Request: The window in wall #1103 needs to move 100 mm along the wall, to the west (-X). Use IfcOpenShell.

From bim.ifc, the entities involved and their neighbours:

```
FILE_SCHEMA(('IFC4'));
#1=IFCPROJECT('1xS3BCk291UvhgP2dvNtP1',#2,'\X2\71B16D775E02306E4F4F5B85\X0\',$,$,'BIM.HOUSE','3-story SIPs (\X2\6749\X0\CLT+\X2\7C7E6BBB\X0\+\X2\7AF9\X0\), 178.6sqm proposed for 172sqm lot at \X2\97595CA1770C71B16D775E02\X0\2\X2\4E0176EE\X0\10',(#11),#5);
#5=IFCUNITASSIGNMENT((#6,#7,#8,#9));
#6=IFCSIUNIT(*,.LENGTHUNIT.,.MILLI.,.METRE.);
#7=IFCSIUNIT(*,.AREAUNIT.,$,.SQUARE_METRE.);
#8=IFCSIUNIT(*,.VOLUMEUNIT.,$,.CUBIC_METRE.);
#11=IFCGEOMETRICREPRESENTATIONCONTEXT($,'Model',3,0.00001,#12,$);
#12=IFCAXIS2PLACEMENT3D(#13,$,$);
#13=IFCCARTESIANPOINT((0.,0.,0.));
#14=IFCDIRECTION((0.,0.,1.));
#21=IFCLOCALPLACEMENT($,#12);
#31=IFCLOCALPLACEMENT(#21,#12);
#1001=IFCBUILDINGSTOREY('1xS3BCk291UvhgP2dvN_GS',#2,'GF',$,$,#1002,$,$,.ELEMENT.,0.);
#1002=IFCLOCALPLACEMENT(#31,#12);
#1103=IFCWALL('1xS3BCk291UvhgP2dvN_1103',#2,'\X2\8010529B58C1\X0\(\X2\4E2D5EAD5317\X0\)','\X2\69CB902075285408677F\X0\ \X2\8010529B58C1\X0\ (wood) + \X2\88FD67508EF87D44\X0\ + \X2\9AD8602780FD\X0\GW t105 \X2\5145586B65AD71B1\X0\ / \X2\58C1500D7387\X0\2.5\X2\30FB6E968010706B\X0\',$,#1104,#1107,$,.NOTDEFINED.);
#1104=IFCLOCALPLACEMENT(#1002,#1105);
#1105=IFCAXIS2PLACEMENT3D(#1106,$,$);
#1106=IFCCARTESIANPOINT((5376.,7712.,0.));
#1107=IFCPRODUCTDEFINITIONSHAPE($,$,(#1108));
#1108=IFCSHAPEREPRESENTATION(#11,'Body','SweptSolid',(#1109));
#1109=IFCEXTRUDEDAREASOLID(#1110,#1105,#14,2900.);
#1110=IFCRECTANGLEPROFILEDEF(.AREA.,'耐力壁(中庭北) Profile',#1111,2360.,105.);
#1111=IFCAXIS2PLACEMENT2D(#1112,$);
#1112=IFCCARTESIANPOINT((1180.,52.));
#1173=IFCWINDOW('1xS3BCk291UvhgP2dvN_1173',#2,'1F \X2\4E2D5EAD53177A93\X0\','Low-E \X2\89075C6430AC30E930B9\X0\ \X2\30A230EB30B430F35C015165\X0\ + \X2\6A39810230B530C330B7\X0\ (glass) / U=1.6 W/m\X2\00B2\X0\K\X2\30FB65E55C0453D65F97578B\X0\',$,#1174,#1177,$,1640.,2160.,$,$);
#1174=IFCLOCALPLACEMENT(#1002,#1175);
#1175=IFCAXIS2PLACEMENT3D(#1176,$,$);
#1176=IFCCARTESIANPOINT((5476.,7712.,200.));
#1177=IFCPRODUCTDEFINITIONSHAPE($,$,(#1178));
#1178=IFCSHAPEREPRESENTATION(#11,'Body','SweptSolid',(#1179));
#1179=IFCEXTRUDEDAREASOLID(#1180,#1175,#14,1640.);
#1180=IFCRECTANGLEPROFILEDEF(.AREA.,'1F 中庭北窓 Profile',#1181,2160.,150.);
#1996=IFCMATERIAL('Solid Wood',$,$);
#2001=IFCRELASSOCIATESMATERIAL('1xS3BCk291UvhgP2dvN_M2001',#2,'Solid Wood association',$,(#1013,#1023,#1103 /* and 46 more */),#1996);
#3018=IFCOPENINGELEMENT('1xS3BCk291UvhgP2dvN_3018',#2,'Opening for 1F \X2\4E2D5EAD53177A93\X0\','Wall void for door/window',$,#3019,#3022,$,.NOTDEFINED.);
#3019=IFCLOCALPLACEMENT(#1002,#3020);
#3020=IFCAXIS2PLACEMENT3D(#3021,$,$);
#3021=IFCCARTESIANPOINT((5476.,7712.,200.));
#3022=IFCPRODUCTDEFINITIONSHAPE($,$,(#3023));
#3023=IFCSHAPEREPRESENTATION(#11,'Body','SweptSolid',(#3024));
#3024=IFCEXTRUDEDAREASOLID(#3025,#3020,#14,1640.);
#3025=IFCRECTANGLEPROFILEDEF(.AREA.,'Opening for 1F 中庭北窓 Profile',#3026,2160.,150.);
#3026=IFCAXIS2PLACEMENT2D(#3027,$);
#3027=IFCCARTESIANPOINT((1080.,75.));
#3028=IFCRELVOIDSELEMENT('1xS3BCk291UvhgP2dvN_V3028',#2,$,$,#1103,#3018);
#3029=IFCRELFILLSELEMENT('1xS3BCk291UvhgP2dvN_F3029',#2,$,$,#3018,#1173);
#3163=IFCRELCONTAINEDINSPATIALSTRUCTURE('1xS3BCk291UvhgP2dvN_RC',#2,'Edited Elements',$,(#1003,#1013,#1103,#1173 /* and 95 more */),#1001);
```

```python
import ifcopenshell
import ifcopenshell.api.geometry
import ifcopenshell.util.placement
import ifcopenshell.util.unit

model = ifcopenshell.open("bim.ifc")
unit_scale = ifcopenshell.util.unit.calculate_unit_scale(model)

window = model.by_guid("1xS3BCk291UvhgP2dvN_1173")
opening = window.FillsVoids[0].RelatingOpeningElement
wall = opening.VoidsElements[0].RelatingBuildingElement

wall_matrix = ifcopenshell.util.placement.get_local_placement(wall.ObjectPlacement)
shift = wall_matrix[:3, 0] * -0.1 / unit_scale
before = ifcopenshell.util.placement.get_local_placement(window.ObjectPlacement)[:3, 3].copy()

# The window is not placed relative to its opening, so move both.
for product in (opening, window):
    matrix = ifcopenshell.util.placement.get_local_placement(product.ObjectPlacement)
    matrix[:3, 3] += shift
    ifcopenshell.api.geometry.edit_object_placement(model, product=product, matrix=matrix, is_si=False)

after = ifcopenshell.util.placement.get_local_placement(window.ObjectPlacement)[:3, 3]
print("window moved by", (after - before).round(3) + 0.0)

model.write("bim_updated.ifc")
```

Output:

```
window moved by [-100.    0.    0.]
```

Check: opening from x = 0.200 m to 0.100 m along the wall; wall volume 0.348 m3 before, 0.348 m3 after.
